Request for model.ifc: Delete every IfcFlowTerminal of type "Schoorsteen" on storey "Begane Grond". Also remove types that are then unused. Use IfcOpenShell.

First a look at what the model holds.

```python
import ifcopenshell
import ifcopenshell.util.element

model = ifcopenshell.open("model.ifc")
print(model.schema)
storey = next(s for s in model.by_type("IfcBuildingStorey") if s.Name == "Begane Grond")
terminals = [e for e in ifcopenshell.util.element.get_decomposition(storey) if e.is_a("IfcFlowTerminal")]
seen = {}
for e in terminals:
    element_type = ifcopenshell.util.element.get_type(e)
    name = element_type.Name if element_type not in (None, e) else None
    seen[name] = seen.get(name, 0) + 1
for name, count in sorted(seen.items(), key=str):
    print(count, "x", name)
```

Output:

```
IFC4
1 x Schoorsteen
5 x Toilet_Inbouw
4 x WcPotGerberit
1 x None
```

```python
import ifcopenshell
import ifcopenshell.api.root
import ifcopenshell.util.element

model = ifcopenshell.open("model.ifc")

storey = next(s for s in model.by_type("IfcBuildingStorey") if s.Name == "Begane Grond")
terminals = [e for e in ifcopenshell.util.element.get_decomposition(storey) if e.is_a("IfcFlowTerminal")]
targets = [e for e in terminals if (t := ifcopenshell.util.element.get_type(e)) not in (None, e) and t.Name == "Schoorsteen"]
types = {ifcopenshell.util.element.get_type(e) for e in targets} - {None, *targets}

for e in targets:
    ifcopenshell.api.root.remove_product(model, product=e)
print(len(targets), "removed")

unused = [t for t in types if not ifcopenshell.util.element.get_types(t)]
for t in unused:
    ifcopenshell.api.root.remove_product(model, product=t)
print(len(unused), "unused types removed")

model.write("model_v2.ifc")
```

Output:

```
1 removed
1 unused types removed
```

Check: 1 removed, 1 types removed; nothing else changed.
